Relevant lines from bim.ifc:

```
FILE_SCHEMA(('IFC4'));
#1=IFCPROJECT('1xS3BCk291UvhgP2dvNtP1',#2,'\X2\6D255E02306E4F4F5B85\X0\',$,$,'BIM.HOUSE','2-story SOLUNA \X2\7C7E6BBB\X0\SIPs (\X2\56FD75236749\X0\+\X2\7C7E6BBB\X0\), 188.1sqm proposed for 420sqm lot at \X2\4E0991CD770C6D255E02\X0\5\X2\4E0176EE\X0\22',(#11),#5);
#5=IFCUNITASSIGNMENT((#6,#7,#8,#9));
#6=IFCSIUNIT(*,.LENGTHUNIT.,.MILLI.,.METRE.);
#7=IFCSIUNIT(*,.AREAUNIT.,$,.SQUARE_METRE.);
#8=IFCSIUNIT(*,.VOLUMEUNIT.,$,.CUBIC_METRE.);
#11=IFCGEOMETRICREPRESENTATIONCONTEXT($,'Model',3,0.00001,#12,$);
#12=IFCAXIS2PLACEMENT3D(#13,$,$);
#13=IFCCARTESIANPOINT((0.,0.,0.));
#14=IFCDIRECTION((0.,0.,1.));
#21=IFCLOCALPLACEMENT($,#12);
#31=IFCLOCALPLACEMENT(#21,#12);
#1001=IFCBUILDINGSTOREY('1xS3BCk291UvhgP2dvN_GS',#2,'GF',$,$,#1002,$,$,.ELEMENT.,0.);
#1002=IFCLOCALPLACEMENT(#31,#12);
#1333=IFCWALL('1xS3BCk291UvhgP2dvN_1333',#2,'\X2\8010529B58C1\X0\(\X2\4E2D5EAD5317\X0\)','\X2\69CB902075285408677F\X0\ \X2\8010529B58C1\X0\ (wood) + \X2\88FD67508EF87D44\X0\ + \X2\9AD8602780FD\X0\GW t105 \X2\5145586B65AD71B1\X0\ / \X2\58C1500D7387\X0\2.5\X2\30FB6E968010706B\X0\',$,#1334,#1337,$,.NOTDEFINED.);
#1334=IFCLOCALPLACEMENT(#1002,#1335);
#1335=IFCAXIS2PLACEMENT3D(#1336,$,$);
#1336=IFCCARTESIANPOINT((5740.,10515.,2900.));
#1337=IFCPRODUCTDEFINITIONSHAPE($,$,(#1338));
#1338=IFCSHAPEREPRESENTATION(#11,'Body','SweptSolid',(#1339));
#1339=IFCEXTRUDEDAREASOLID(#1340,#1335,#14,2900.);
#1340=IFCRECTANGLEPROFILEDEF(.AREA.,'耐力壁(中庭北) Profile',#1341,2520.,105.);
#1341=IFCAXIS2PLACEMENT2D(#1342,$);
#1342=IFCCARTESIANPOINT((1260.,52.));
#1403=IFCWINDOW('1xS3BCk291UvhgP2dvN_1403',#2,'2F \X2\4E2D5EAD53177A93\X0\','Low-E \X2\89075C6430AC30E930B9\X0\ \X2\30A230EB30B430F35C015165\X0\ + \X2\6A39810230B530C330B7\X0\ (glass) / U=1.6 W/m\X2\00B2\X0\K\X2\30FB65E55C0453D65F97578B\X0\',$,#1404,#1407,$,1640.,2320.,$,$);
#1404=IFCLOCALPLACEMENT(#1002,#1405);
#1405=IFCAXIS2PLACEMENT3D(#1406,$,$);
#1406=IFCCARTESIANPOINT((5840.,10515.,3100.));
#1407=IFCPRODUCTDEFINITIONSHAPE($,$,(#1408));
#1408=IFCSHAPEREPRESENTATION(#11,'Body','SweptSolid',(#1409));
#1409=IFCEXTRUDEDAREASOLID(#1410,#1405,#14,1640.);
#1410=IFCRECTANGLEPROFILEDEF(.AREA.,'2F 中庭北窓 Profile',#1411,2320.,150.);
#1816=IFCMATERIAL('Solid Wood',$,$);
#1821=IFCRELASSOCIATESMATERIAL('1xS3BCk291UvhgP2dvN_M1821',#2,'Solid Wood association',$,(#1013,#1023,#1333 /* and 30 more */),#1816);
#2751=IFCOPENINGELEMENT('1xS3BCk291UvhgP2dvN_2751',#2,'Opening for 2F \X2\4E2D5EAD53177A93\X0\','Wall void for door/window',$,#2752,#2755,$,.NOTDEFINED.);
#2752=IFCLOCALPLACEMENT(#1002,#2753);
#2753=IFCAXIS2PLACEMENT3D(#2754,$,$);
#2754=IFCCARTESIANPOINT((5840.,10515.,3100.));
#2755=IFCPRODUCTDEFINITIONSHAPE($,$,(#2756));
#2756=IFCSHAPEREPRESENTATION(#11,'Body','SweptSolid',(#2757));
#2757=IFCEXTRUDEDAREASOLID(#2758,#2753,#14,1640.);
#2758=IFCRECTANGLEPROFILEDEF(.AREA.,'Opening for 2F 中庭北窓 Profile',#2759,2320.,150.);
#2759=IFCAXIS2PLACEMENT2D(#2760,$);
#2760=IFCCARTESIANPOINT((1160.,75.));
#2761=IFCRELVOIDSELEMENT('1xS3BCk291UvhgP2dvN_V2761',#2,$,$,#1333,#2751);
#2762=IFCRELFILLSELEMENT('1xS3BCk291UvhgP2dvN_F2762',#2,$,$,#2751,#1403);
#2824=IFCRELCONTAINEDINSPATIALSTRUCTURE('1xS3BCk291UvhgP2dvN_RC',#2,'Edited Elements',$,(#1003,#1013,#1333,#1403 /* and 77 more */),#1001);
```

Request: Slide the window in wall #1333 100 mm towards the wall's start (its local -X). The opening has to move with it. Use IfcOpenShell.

```python
import ifcopenshell
import ifcopenshell.api.geometry
import ifcopenshell.util.placement
import ifcopenshell.util.unit

model = ifcopenshell.open("bim.ifc")
unit_scale = ifcopenshell.util.unit.calculate_unit_scale(model)

window = model.by_guid("1xS3BCk291UvhgP2dvN_1403")
opening = window.FillsVoids[0].RelatingOpeningElement
wall = opening.VoidsElements[0].RelatingBuildingElement

wall_matrix = ifcopenshell.util.placement.get_local_placement(wall.ObjectPlacement)
shift = wall_matrix[:3, 0] * -0.1 / unit_scale
before = ifcopenshell.util.placement.get_local_placement(window.ObjectPlacement)[:3, 3].copy()

# The window is not placed relative to its opening, so move both.
for product in (opening, window):
    matrix = ifcopenshell.util.placement.get_local_placement(product.ObjectPlacement)
    matrix[:3, 3] += shift
    ifcopenshell.api.geometry.edit_object_placement(model, product=product, matrix=matrix, is_si=False)

after = ifcopenshell.util.placement.get_local_placement(window.ObjectPlacement)[:3, 3]
print("window moved by", (after - before).round(3) + 0.0)

model.write("bim_rev.ifc")
```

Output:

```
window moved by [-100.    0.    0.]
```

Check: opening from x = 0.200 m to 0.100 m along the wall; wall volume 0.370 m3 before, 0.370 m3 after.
